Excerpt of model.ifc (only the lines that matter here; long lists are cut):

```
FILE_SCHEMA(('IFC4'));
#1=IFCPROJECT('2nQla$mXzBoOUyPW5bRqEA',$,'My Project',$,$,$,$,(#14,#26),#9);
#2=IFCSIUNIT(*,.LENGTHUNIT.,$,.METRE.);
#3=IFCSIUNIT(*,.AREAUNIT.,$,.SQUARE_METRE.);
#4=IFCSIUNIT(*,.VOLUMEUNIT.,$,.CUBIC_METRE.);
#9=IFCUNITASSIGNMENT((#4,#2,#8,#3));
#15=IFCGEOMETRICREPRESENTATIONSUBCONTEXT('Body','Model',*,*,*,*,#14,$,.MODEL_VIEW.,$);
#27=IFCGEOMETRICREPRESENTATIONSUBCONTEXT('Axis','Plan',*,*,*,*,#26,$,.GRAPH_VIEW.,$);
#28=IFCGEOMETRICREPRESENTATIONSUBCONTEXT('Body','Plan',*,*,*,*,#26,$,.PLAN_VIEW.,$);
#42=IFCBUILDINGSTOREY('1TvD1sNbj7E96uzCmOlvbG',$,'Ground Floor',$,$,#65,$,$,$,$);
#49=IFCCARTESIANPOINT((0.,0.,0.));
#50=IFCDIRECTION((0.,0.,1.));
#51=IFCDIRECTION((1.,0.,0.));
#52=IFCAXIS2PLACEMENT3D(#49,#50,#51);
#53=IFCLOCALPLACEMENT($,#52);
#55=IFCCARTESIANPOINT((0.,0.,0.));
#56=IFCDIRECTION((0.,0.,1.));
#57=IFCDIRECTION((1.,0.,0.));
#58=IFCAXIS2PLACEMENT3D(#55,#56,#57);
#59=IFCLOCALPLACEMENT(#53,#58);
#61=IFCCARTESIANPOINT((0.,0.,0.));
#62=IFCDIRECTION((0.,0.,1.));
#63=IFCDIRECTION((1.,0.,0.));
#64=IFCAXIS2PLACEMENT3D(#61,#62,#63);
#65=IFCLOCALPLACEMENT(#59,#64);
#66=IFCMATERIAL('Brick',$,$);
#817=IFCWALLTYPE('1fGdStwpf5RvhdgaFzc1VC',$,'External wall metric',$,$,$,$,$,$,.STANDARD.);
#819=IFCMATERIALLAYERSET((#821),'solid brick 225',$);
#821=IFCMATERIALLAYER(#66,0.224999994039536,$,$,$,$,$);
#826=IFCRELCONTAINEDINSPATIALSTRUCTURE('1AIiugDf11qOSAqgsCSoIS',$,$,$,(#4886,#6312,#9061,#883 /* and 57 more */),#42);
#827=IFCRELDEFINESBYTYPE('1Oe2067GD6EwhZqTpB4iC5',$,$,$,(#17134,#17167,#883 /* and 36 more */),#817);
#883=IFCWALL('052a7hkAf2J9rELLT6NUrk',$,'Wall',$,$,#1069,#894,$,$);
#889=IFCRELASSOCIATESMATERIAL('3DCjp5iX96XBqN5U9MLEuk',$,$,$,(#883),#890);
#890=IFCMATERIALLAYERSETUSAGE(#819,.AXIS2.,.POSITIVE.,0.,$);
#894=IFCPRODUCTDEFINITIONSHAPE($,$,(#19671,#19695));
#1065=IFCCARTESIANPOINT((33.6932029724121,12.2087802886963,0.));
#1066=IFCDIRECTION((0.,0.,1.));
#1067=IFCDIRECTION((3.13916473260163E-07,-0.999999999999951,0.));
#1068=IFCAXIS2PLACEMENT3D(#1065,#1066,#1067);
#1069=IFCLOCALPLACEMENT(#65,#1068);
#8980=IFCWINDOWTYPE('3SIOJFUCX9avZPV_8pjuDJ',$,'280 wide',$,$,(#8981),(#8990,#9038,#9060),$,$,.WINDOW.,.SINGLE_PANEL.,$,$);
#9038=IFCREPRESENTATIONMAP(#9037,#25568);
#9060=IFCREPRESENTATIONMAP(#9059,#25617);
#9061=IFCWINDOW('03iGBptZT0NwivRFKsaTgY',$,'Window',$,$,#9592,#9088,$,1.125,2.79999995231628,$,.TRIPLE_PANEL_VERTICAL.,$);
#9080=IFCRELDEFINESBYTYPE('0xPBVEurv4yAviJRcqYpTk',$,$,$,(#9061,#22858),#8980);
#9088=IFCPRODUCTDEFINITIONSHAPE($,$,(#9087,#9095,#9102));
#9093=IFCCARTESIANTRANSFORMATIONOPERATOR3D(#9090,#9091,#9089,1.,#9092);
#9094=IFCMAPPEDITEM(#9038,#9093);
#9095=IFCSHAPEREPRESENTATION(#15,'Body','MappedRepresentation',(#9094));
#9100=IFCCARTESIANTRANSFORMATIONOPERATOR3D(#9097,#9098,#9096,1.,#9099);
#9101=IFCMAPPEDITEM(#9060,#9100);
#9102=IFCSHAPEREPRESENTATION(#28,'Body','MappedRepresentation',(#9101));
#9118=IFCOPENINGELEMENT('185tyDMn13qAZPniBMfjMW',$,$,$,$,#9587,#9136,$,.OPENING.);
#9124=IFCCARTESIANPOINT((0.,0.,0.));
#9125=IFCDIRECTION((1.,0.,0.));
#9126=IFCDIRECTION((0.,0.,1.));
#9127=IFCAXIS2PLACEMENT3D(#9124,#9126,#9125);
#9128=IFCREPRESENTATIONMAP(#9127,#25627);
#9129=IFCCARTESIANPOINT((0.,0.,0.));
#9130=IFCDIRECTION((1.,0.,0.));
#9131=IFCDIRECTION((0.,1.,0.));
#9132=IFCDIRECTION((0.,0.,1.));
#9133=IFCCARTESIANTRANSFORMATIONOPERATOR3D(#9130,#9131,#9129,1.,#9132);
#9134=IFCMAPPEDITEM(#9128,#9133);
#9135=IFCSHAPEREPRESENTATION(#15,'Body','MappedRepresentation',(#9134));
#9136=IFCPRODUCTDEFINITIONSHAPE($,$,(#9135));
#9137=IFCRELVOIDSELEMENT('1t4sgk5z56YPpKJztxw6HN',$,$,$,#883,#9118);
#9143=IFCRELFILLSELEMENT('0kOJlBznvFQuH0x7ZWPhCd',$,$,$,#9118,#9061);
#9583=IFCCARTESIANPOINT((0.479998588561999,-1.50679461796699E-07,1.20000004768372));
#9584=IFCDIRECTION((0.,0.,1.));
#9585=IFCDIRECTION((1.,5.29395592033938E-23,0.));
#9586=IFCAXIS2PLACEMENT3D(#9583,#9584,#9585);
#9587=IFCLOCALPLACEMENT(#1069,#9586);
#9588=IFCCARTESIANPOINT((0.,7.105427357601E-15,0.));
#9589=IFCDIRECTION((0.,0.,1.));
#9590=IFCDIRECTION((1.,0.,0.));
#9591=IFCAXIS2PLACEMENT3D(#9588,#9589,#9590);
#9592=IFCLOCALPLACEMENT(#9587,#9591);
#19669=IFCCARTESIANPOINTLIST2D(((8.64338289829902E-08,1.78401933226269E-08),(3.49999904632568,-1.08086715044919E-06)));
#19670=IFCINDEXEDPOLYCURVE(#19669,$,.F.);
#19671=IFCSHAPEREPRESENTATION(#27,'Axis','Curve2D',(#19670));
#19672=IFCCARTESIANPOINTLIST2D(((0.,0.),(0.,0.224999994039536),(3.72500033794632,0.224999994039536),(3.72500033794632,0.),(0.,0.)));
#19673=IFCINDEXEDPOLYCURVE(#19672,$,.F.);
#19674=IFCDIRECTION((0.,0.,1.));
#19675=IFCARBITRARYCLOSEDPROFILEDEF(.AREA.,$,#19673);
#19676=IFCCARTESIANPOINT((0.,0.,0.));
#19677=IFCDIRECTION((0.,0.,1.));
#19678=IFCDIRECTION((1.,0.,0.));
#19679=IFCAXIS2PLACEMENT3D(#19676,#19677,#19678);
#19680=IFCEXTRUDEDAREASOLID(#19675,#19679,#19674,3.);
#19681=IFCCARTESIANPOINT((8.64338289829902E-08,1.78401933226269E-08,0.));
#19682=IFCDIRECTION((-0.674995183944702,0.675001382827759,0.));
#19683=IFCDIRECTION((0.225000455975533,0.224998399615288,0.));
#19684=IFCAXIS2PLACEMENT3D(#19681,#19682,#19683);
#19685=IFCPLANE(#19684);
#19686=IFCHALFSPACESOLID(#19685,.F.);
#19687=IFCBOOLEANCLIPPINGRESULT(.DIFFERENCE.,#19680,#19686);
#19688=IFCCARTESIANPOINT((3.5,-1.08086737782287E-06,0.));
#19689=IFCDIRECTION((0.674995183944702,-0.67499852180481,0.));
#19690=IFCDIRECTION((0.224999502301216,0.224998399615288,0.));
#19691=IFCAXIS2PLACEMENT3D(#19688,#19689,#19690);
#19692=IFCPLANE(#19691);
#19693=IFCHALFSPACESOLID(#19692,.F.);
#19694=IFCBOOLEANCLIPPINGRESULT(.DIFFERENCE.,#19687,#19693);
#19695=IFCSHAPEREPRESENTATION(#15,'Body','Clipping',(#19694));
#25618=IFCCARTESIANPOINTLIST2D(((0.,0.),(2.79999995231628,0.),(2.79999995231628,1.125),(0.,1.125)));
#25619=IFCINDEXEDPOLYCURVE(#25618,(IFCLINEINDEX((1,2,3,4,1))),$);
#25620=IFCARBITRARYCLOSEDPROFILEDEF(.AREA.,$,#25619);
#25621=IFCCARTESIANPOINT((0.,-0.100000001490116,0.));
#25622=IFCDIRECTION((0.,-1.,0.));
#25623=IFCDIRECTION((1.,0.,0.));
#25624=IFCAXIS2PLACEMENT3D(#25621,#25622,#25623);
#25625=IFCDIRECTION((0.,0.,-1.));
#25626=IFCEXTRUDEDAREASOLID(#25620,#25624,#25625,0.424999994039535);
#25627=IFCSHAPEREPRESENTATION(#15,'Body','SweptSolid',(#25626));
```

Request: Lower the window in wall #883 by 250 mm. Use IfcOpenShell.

```python
import numpy as np
import ifcopenshell
import ifcopenshell.api.geometry
import ifcopenshell.util.placement
import ifcopenshell.util.unit

model = ifcopenshell.open("model.ifc")
unit_scale = ifcopenshell.util.unit.calculate_unit_scale(model)

window = model.by_guid("03iGBptZT0NwivRFKsaTgY")
opening = window.FillsVoids[0].RelatingOpeningElement
dz = -0.25

shift = np.array([0.0, 0.0, dz])
# The window is placed relative to its opening, so it follows when the opening moves.
matrix = ifcopenshell.util.placement.get_local_placement(opening.ObjectPlacement)
matrix[:3, 3] += shift
ifcopenshell.api.geometry.edit_object_placement(
    model, product=opening, matrix=matrix, is_si=False, should_transform_children=True
)

print(f"moved by {dz * unit_scale:+.3f} m")

model.write("model_v2.ifc")
```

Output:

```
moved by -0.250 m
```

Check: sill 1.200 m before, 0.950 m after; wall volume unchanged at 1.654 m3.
